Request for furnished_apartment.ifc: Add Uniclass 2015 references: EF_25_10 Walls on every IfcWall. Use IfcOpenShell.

First a look at what the model holds.

```python
import ifcopenshell

model = ifcopenshell.open("furnished_apartment.ifc")
print(model.schema)
print("classifications:", [c.Name for c in model.by_type("IfcClassification")])
for ifc_class in ("IfcDoor", "IfcRoof", "IfcStair", "IfcWall", "IfcWindow"):
    print(ifc_class, len(model.by_type(ifc_class)))
```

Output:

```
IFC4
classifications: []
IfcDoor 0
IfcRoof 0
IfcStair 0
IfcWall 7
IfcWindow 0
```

```python
import ifcopenshell
import ifcopenshell.api.classification

model = ifcopenshell.open("furnished_apartment.ifc")

system = ifcopenshell.api.classification.add_classification(model, classification="Uniclass 2015")

codes = {
    "IfcWall": ("EF_25_10", "Walls"),
}
for ifc_class, (code, name) in codes.items():
    products = model.by_type(ifc_class)
    ifcopenshell.api.classification.add_reference(
        model, products=products, classification=system, identification=code, name=name
    )
    print(code, len(products))

model.write("furnished_apartment_v2.ifc")
```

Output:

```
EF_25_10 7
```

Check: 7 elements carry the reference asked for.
